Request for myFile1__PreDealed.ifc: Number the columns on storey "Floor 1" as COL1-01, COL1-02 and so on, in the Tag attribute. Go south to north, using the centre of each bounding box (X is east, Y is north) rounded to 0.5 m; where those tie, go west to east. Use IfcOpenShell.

First a look at what the model holds.

```python
import ifcopenshell
import ifcopenshell.util.element
import ifcopenshell.util.placement

model = ifcopenshell.open("myFile1__PreDealed.ifc")
print(model.schema)
storey = next(s for s in model.by_type("IfcBuildingStorey") if s.Name == "Floor 1")
columns = [e for e in ifcopenshell.util.element.get_decomposition(storey) if e.is_a("IfcColumn")]
for e in sorted(columns, key=lambda e: e.id()):
    origin = ifcopenshell.util.placement.get_local_placement(e.ObjectPlacement)[:3, 3]
    print(e.id(), e.Tag, e.Name, origin.round(2) + 0.0, sep=" | ")
```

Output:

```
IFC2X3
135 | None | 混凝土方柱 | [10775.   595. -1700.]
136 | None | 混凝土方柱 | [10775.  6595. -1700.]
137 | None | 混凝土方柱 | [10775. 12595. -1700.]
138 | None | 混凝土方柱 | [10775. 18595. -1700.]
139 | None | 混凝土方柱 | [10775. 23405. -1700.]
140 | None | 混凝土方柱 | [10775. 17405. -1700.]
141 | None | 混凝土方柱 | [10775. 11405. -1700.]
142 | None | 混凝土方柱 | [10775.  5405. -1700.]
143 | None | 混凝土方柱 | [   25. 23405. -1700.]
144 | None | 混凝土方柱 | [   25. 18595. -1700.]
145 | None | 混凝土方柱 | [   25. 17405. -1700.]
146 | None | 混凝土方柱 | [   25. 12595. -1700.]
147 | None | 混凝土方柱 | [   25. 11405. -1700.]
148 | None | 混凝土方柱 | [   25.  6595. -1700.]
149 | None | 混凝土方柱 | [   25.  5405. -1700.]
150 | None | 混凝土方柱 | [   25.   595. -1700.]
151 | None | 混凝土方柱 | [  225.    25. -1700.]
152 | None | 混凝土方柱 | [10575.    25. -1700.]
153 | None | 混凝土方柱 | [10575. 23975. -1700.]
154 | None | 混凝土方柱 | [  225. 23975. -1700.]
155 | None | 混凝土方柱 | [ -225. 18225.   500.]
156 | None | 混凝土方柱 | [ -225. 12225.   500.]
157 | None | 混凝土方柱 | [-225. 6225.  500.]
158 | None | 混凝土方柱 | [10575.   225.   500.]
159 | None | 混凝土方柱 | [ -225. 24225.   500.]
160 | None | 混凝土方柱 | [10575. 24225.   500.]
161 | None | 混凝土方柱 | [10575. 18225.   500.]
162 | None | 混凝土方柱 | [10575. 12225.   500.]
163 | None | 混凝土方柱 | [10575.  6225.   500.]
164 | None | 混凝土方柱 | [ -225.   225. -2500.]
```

```python
import ifcopenshell
import ifcopenshell.geom
import ifcopenshell.util.element
import ifcopenshell.util.shape

model = ifcopenshell.open("myFile1__PreDealed.ifc")
settings = ifcopenshell.geom.settings()
settings.set("use-world-coords", True)


def centre(element):
    shape = ifcopenshell.geom.create_shape(settings, element)
    return ifcopenshell.util.shape.get_bbox_centroid(shape.geometry)


storey = next(s for s in model.by_type("IfcBuildingStorey") if s.Name == "Floor 1")
columns = [e for e in ifcopenshell.util.element.get_decomposition(storey) if e.is_a("IfcColumn")]

# Insertion points can sit at a corner or the storey origin, so sort by the geometry (in metres).
centres = {e: centre(e) for e in columns}
columns.sort(key=lambda e: (round(centres[e][1] / 0.5), centres[e][0]))

for i, e in enumerate(columns, start=1):
    number = f"COL1-{i:02d}"
    e.Tag = number
    print(e.id(), number)

model.write("myFile1__PreDealed_updated.ifc")
```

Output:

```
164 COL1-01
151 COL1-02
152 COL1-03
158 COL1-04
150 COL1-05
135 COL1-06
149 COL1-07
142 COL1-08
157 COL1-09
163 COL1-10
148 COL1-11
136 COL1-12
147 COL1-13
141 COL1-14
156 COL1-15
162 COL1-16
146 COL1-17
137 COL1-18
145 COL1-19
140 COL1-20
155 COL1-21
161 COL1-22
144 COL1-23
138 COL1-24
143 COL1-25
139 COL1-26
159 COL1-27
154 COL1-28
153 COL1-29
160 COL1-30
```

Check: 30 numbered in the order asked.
